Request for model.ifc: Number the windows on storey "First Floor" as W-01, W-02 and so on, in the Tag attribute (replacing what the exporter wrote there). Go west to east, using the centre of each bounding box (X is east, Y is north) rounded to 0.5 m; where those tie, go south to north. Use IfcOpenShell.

First a look at what the model holds.

```python
import ifcopenshell
import ifcopenshell.util.element
import ifcopenshell.util.placement

model = ifcopenshell.open("model.ifc")
print(model.schema)
storey = next(s for s in model.by_type("IfcBuildingStorey") if s.Name == "First Floor")
windows = [e for e in ifcopenshell.util.element.get_decomposition(storey) if e.is_a("IfcWindow")]
for e in sorted(windows, key=lambda e: e.id()):
    origin = ifcopenshell.util.placement.get_local_placement(e.ObjectPlacement)[:3, 3]
    print(e.id(), e.Tag, e.Name, origin.round(2) + 0.0, sep=" | ")
```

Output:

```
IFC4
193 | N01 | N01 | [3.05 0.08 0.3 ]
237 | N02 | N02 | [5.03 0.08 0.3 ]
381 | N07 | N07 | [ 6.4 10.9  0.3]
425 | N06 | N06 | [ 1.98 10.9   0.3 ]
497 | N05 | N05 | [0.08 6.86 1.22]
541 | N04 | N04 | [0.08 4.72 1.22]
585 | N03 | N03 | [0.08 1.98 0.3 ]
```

```python
import ifcopenshell
import ifcopenshell.geom
import ifcopenshell.util.element
import ifcopenshell.util.shape

model = ifcopenshell.open("model.ifc")
settings = ifcopenshell.geom.settings()
settings.set("use-world-coords", True)


def centre(element):
    shape = ifcopenshell.geom.create_shape(settings, element)
    return ifcopenshell.util.shape.get_bbox_centroid(shape.geometry)


storey = next(s for s in model.by_type("IfcBuildingStorey") if s.Name == "First Floor")
windows = [e for e in ifcopenshell.util.element.get_decomposition(storey) if e.is_a("IfcWindow")]

# Insertion points can sit at a corner or the storey origin, so sort by the geometry (in metres).
centres = {e: centre(e) for e in windows}
windows.sort(key=lambda e: (round(centres[e][0] / 0.5), centres[e][1]))

for i, e in enumerate(windows, start=1):
    number = f"W-{i:02d}"
    e.Tag = number
    print(e.id(), number)

model.write("model_updated.ifc")
```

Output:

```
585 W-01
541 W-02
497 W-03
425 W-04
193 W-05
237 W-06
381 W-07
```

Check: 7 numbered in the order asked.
